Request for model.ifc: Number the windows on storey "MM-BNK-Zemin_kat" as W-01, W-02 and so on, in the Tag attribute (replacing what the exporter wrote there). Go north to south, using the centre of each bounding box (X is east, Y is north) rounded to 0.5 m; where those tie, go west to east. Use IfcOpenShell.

First a look at what the model holds.

```python
import ifcopenshell
import ifcopenshell.util.element
import ifcopenshell.util.placement

model = ifcopenshell.open("model.ifc")
print(model.schema)
storey = next(s for s in model.by_type("IfcBuildingStorey") if s.Name == "MM-BNK-Zemin_kat")
windows = [e for e in ifcopenshell.util.element.get_decomposition(storey) if e.is_a("IfcWindow")]
for e in sorted(windows, key=lambda e: e.id()):
    origin = ifcopenshell.util.placement.get_local_placement(e.ObjectPlacement)[:3, 3]
    print(e.id(), e.Tag, e.Name, origin.round(2) + 0.0, sep=" | ")
```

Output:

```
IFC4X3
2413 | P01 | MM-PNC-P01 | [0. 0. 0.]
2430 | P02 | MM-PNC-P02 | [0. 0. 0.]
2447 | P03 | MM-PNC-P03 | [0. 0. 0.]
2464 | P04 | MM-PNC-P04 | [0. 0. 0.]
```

```python
import ifcopenshell
import ifcopenshell.geom
import ifcopenshell.util.element
import ifcopenshell.util.shape

model = ifcopenshell.open("model.ifc")
settings = ifcopenshell.geom.settings()
settings.set("use-world-coords", True)


def centre(element):
    shape = ifcopenshell.geom.create_shape(settings, element)
    return ifcopenshell.util.shape.get_bbox_centroid(shape.geometry)


storey = next(s for s in model.by_type("IfcBuildingStorey") if s.Name == "MM-BNK-Zemin_kat")
windows = [e for e in ifcopenshell.util.element.get_decomposition(storey) if e.is_a("IfcWindow")]

# Insertion points can sit at a corner or the storey origin, so sort by the geometry (in metres).
centres = {e: centre(e) for e in windows}
windows.sort(key=lambda e: (-round(centres[e][1] / 0.5), centres[e][0]))

for i, e in enumerate(windows, start=1):
    number = f"W-{i:02d}"
    e.Tag = number
    print(e.id(), number)

model.write("model-out.ifc")
```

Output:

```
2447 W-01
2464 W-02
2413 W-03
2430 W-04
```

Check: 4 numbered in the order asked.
